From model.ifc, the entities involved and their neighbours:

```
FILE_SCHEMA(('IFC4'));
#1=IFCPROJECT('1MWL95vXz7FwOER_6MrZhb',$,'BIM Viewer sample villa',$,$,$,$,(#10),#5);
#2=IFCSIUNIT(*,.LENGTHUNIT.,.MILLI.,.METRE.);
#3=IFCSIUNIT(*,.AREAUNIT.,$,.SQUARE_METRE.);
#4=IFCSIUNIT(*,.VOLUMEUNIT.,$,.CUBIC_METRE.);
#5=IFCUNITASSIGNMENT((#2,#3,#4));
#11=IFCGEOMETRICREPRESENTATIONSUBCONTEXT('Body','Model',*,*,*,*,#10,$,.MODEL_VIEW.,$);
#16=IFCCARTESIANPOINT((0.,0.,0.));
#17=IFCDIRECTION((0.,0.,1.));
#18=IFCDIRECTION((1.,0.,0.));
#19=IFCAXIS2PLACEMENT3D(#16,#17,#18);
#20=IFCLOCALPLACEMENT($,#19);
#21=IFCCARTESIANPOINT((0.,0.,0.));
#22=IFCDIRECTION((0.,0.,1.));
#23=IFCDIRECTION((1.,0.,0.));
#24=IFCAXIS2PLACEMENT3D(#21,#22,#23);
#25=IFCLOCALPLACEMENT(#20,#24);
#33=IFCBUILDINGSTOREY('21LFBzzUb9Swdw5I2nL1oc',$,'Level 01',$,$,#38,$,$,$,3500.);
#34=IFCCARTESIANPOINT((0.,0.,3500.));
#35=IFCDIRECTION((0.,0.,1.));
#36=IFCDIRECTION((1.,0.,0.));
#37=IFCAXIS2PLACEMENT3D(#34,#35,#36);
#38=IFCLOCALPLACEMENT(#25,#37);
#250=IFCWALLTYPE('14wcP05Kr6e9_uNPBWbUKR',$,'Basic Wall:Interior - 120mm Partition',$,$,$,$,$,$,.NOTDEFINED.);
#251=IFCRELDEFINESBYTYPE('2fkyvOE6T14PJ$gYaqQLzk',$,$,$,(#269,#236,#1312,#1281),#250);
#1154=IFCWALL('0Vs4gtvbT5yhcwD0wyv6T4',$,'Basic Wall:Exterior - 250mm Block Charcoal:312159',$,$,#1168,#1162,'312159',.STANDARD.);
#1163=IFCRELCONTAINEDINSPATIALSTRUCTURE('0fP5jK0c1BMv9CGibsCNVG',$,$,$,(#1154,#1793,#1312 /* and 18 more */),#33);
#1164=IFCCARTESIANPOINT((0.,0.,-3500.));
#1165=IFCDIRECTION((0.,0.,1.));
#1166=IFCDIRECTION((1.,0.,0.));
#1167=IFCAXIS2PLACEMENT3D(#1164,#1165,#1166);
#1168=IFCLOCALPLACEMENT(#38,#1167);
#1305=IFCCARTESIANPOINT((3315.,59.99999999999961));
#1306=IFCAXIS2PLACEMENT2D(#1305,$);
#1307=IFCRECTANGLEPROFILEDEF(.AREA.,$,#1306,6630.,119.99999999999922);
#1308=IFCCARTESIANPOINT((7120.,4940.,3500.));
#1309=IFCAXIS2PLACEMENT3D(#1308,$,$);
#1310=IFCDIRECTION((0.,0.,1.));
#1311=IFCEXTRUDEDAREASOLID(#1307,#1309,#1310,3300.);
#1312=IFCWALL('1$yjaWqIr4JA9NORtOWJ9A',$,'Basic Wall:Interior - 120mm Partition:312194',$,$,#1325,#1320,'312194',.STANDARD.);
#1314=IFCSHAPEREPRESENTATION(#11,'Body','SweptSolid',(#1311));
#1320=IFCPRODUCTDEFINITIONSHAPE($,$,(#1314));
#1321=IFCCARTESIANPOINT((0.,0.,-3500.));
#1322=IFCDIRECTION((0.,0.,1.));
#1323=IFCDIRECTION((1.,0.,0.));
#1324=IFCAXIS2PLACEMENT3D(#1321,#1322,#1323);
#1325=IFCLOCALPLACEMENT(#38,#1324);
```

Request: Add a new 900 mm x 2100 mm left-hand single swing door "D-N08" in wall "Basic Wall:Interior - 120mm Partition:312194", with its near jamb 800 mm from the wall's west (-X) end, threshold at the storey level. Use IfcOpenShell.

```python
import numpy as np
import ifcopenshell
import ifcopenshell.api.feature
import ifcopenshell.api.geometry
import ifcopenshell.api.root
import ifcopenshell.api.spatial
import ifcopenshell.geom
import ifcopenshell.util.element
import ifcopenshell.util.placement
import ifcopenshell.util.representation
import ifcopenshell.util.shape
import ifcopenshell.util.unit

model = ifcopenshell.open("model.ifc")
unit_scale = ifcopenshell.util.unit.calculate_unit_scale(model)
settings = ifcopenshell.geom.settings()


def volume(element):
    """Net volume in cubic metres, openings subtracted."""
    shape = ifcopenshell.geom.create_shape(settings, element)
    return ifcopenshell.util.shape.get_volume(shape.geometry)


wall = model.by_guid("1$yjaWqIr4JA9NORtOWJ9A")
storey = ifcopenshell.util.element.get_container(wall, ifc_class="IfcBuildingStorey")
context = ifcopenshell.util.representation.get_context(model, "Model", "Body", "MODEL_VIEW")
before = volume(wall)

width, height, from_end, sill = 0.9, 2.1, 0.8, 0.0  # metres

# The wall runs along its own X axis, and the end named is its -X end.
wall_shape = ifcopenshell.geom.create_shape(settings, wall)
x, y, z = ifcopenshell.util.shape.get_vertices(wall_shape.geometry).T
start = x.min() + from_end
face, thickness = float(y.min()), float(y.max() - y.min())
wall_matrix = ifcopenshell.util.placement.get_local_placement(wall.ObjectPlacement)
level = ifcopenshell.util.placement.get_local_placement(storey.ObjectPlacement)[2, 3]


def in_wall(x, y):
    """Placement at x, y metres in the wall's axes, at sill height."""
    matrix = wall_matrix.copy()
    matrix[:, 3] = wall_matrix @ np.array([x / unit_scale, y / unit_scale, 0.0, 1.0])
    matrix[2, 3] = level + sill / unit_scale
    return matrix


# Opening: a box that overshoots both wall faces by 50 mm.
opening = ifcopenshell.api.root.create_entity(model, ifc_class="IfcOpeningElement", predefined_type="OPENING")
box = ifcopenshell.api.geometry.add_wall_representation(
    model, context=context, length=width, height=height, thickness=thickness + 0.1
)
ifcopenshell.api.geometry.assign_representation(model, product=opening, representation=box)
ifcopenshell.api.geometry.edit_object_placement(model, product=opening, matrix=in_wall(start, face - 0.05), is_si=False)
ifcopenshell.api.feature.add_feature(model, feature=opening, element=wall)

door = ifcopenshell.api.root.create_entity(model, ifc_class="IfcDoor", name="D-N08", predefined_type="DOOR")
door.OverallWidth, door.OverallHeight = width / unit_scale, height / unit_scale
door.OperationType = "SINGLE_SWING_LEFT"
body = ifcopenshell.api.geometry.add_door_representation(
    model,
    context=context,
    overall_width=door.OverallWidth,
    overall_height=door.OverallHeight,
    operation_type="SINGLE_SWING_LEFT",
    lining_properties={"LiningDepth": thickness / unit_scale, "ThresholdDepth": thickness / unit_scale},
)
ifcopenshell.api.geometry.assign_representation(model, product=door, representation=body)
ifcopenshell.api.spatial.assign_container(model, products=[door], relating_structure=storey)
ifcopenshell.api.feature.add_filling(model, opening=opening, element=door)

# The lining spans the wall, so the door starts at the wall face.
ifcopenshell.api.geometry.edit_object_placement(model, product=door, matrix=in_wall(start, face), is_si=False)

after = volume(wall)

print(f"wall volume {before:.3f} -> {after:.3f} m3")

model.write("model_updated.ifc")
```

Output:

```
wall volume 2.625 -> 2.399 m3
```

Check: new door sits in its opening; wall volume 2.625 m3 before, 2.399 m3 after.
